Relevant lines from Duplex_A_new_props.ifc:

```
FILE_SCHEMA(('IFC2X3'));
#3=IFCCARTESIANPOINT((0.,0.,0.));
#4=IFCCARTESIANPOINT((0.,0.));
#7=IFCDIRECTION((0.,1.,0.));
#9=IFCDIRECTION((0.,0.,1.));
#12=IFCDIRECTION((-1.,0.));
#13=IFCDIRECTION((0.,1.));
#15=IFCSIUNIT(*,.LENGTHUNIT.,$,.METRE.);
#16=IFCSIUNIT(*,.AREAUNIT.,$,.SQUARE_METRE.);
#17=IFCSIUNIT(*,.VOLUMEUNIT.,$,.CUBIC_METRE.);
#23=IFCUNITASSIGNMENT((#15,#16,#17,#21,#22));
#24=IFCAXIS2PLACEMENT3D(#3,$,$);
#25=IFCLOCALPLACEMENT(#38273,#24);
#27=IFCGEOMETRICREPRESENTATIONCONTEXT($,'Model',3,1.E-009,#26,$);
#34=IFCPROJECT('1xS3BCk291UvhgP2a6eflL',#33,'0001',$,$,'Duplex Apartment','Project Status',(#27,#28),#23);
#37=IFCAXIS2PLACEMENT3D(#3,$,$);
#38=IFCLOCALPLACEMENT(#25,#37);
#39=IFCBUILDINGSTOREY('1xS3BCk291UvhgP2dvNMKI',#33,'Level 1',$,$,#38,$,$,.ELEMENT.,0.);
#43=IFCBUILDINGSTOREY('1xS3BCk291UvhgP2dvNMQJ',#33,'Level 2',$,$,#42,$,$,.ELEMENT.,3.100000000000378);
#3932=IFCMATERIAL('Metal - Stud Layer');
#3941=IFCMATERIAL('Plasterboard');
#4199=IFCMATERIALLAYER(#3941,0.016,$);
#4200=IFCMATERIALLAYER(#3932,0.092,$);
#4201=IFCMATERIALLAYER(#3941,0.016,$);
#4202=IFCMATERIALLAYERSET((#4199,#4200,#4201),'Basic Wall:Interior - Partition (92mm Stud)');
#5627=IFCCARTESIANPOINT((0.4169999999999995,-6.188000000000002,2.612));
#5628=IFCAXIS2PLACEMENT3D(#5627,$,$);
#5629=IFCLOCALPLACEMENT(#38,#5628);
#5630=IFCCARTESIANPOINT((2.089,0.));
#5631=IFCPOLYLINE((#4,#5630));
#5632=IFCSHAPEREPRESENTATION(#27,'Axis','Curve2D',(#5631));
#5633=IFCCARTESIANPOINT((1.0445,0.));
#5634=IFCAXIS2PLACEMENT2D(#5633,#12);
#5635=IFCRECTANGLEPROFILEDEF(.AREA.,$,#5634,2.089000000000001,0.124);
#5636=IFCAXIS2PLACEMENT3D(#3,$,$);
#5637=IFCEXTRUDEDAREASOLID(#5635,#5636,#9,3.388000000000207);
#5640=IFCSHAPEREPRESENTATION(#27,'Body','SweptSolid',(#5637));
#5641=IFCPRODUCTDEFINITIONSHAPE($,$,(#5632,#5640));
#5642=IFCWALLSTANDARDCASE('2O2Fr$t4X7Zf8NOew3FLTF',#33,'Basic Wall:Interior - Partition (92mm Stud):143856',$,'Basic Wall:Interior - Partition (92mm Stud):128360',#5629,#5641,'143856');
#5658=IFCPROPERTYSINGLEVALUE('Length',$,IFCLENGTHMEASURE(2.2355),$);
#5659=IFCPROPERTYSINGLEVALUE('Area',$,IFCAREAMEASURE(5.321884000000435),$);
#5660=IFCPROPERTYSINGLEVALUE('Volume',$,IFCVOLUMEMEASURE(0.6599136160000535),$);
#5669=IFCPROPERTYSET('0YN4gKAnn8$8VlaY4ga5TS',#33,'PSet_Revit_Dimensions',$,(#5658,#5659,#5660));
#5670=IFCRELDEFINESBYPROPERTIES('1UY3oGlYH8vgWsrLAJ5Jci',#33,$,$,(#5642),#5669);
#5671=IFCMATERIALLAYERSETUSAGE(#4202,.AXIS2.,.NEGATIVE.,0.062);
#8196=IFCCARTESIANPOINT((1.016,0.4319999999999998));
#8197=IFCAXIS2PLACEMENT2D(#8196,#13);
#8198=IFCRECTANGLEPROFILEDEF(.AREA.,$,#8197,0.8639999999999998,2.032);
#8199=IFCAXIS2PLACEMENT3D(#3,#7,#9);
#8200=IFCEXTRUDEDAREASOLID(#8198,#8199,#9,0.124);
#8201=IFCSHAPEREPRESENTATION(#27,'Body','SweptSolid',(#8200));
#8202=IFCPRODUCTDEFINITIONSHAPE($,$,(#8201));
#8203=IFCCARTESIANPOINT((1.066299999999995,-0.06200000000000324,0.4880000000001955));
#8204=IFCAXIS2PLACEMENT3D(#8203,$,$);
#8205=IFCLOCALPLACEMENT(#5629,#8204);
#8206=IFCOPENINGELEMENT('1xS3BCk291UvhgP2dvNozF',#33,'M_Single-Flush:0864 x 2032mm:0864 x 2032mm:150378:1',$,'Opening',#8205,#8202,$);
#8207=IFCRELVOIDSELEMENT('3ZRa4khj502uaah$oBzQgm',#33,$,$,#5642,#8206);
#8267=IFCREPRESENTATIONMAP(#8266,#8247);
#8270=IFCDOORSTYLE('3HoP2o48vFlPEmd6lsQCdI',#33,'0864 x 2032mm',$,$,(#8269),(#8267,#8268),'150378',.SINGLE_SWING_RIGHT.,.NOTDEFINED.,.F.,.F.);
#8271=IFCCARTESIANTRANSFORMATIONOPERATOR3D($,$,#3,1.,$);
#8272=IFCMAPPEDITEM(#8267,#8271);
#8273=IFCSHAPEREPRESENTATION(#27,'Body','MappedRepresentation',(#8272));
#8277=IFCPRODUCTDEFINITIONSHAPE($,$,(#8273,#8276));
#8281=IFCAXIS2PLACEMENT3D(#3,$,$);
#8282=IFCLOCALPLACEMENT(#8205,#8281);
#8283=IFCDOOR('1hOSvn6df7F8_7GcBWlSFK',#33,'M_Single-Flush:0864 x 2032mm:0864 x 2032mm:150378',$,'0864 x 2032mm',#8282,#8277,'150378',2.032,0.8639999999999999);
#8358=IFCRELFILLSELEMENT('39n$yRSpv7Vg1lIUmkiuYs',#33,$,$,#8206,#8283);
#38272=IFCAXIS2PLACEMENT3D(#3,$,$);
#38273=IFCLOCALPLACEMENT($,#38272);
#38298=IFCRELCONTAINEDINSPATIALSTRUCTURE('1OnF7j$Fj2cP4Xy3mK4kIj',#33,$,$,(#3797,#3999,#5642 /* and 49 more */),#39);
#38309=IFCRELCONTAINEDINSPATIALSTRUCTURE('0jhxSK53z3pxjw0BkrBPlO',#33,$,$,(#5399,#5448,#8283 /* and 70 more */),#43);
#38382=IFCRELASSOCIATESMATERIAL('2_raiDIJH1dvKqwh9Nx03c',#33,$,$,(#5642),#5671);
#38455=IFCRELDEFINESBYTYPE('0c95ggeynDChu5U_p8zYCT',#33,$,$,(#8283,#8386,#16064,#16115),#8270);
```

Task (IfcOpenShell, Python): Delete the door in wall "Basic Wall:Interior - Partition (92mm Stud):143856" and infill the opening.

```python
import ifcopenshell
import ifcopenshell.api.feature
import ifcopenshell.api.pset
import ifcopenshell.api.root
import ifcopenshell.geom
import ifcopenshell.util.element
import ifcopenshell.util.shape
import ifcopenshell.util.unit

model = ifcopenshell.open("Duplex_A_new_props.ifc")
area_scale = ifcopenshell.util.unit.calculate_unit_scale(model, "AREAUNIT")
volume_scale = ifcopenshell.util.unit.calculate_unit_scale(model, "VOLUMEUNIT")
settings = ifcopenshell.geom.settings()


def volume(element):
    """Net volume in cubic metres, openings subtracted."""
    shape = ifcopenshell.geom.create_shape(settings, element)
    return ifcopenshell.util.shape.get_volume(shape.geometry)


door = model.by_id(8283)
opening = door.FillsVoids[0].RelatingOpeningElement
wall = opening.VoidsElements[0].RelatingBuildingElement
before = volume(wall)

ifcopenshell.api.root.remove_product(model, product=door)
ifcopenshell.api.feature.remove_feature(model, feature=opening)

after = volume(wall)
thickness = 0.124  # wall thickness in metres

# Update the wall's stored quantities.
pset = model.by_id(ifcopenshell.util.element.get_pset(wall, "PSet_Revit_Dimensions", should_inherit=False)["id"])
ifcopenshell.api.pset.edit_pset(model, pset=pset, properties={
    "Area": model.create_entity("IfcAreaMeasure", after / thickness / area_scale),
    "Volume": model.create_entity("IfcVolumeMeasure", after / volume_scale),
})

print(f"wall volume {before:.3f} -> {after:.3f} m3")

model.write("Duplex_A_new_props_v2.ifc")
```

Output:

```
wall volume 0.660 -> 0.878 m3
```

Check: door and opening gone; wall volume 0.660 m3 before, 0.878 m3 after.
